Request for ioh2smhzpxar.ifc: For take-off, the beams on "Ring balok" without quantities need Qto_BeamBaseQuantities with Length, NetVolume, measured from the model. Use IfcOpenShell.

First a look at what the model holds.

```python
import ifcopenshell
import ifcopenshell.util.element
import ifcopenshell.util.unit

model = ifcopenshell.open("ioh2smhzpxar.ifc")
print(model.schema)
for unit_type in ("LENGTHUNIT", "AREAUNIT", "VOLUMEUNIT"):
    print(unit_type, ifcopenshell.util.unit.calculate_unit_scale(model, unit_type))
storey = next(s for s in model.by_type("IfcBuildingStorey") if s.Name == "Ring balok")
beams = [e for e in ifcopenshell.util.element.get_decomposition(storey) if e.is_a("IfcBeam")]
for e in sorted(beams, key=lambda e: e.id()):
    print(e.id(), e.is_a(), e.Name, list(ifcopenshell.util.element.get_psets(e, qtos_only=True)), sep=" | ")
```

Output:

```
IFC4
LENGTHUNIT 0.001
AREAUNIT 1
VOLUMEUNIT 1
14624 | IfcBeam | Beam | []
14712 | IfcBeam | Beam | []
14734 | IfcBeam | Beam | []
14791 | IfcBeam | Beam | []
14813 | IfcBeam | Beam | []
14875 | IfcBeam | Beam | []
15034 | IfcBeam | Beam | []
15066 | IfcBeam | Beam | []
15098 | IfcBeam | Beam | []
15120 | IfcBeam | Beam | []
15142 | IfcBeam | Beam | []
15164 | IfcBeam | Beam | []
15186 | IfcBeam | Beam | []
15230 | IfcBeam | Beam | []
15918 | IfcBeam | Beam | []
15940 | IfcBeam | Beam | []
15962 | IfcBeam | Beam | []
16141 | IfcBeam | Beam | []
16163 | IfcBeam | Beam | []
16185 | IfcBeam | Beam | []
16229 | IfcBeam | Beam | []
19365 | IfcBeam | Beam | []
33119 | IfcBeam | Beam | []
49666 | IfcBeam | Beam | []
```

```python
import ifcopenshell
import ifcopenshell.api.pset
import ifcopenshell.geom
import ifcopenshell.util.element
import ifcopenshell.util.shape
import ifcopenshell.util.unit

model = ifcopenshell.open("ioh2smhzpxar.ifc")
unit_scale = ifcopenshell.util.unit.calculate_unit_scale(model)
volume_scale = ifcopenshell.util.unit.calculate_unit_scale(model, "VOLUMEUNIT")
settings = ifcopenshell.geom.settings()

storey = next(s for s in model.by_type("IfcBuildingStorey") if s.Name == "Ring balok")
beams = [e for e in ifcopenshell.util.element.get_decomposition(storey) if e.is_a("IfcBeam")]

for e in sorted(beams, key=lambda e: e.id()):
    if ifcopenshell.util.element.get_psets(e, qtos_only=True, should_inherit=False):
        continue
    # Geometry comes back in metres, in the element's own axes.
    shape = ifcopenshell.geom.create_shape(settings, e)
    values = {
        "Length": ifcopenshell.util.shape.get_max_xyz(shape.geometry) / unit_scale,
        "NetVolume": ifcopenshell.util.shape.get_volume(shape.geometry) / volume_scale,
    }
    qto = ifcopenshell.api.pset.add_qto(model, product=e, name="Qto_BeamBaseQuantities")
    ifcopenshell.api.pset.edit_qto(model, qto=qto, properties=values)
    print(e.id(), {k: round(v, 3) for k, v in values.items()})

model.write("ioh2smhzpxar_edited.ifc")
```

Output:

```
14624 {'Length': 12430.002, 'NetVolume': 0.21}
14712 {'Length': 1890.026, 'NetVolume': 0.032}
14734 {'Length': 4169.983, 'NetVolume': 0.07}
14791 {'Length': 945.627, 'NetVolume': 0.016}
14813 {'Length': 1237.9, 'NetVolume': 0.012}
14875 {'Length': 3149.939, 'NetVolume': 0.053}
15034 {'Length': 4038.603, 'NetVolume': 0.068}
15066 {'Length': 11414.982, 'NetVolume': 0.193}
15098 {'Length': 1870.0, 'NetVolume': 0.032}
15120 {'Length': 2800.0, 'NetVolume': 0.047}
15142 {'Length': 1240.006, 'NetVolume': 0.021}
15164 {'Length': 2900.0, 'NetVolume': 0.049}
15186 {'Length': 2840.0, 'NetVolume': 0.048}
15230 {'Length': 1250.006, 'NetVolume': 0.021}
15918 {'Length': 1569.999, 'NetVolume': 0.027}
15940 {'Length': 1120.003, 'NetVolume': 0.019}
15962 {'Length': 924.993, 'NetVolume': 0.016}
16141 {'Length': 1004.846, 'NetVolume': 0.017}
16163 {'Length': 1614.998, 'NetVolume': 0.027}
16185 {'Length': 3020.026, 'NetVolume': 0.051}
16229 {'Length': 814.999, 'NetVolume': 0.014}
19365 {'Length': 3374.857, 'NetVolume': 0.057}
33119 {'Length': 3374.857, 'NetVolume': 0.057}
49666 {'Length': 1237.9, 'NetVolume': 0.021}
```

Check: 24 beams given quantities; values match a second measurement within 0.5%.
